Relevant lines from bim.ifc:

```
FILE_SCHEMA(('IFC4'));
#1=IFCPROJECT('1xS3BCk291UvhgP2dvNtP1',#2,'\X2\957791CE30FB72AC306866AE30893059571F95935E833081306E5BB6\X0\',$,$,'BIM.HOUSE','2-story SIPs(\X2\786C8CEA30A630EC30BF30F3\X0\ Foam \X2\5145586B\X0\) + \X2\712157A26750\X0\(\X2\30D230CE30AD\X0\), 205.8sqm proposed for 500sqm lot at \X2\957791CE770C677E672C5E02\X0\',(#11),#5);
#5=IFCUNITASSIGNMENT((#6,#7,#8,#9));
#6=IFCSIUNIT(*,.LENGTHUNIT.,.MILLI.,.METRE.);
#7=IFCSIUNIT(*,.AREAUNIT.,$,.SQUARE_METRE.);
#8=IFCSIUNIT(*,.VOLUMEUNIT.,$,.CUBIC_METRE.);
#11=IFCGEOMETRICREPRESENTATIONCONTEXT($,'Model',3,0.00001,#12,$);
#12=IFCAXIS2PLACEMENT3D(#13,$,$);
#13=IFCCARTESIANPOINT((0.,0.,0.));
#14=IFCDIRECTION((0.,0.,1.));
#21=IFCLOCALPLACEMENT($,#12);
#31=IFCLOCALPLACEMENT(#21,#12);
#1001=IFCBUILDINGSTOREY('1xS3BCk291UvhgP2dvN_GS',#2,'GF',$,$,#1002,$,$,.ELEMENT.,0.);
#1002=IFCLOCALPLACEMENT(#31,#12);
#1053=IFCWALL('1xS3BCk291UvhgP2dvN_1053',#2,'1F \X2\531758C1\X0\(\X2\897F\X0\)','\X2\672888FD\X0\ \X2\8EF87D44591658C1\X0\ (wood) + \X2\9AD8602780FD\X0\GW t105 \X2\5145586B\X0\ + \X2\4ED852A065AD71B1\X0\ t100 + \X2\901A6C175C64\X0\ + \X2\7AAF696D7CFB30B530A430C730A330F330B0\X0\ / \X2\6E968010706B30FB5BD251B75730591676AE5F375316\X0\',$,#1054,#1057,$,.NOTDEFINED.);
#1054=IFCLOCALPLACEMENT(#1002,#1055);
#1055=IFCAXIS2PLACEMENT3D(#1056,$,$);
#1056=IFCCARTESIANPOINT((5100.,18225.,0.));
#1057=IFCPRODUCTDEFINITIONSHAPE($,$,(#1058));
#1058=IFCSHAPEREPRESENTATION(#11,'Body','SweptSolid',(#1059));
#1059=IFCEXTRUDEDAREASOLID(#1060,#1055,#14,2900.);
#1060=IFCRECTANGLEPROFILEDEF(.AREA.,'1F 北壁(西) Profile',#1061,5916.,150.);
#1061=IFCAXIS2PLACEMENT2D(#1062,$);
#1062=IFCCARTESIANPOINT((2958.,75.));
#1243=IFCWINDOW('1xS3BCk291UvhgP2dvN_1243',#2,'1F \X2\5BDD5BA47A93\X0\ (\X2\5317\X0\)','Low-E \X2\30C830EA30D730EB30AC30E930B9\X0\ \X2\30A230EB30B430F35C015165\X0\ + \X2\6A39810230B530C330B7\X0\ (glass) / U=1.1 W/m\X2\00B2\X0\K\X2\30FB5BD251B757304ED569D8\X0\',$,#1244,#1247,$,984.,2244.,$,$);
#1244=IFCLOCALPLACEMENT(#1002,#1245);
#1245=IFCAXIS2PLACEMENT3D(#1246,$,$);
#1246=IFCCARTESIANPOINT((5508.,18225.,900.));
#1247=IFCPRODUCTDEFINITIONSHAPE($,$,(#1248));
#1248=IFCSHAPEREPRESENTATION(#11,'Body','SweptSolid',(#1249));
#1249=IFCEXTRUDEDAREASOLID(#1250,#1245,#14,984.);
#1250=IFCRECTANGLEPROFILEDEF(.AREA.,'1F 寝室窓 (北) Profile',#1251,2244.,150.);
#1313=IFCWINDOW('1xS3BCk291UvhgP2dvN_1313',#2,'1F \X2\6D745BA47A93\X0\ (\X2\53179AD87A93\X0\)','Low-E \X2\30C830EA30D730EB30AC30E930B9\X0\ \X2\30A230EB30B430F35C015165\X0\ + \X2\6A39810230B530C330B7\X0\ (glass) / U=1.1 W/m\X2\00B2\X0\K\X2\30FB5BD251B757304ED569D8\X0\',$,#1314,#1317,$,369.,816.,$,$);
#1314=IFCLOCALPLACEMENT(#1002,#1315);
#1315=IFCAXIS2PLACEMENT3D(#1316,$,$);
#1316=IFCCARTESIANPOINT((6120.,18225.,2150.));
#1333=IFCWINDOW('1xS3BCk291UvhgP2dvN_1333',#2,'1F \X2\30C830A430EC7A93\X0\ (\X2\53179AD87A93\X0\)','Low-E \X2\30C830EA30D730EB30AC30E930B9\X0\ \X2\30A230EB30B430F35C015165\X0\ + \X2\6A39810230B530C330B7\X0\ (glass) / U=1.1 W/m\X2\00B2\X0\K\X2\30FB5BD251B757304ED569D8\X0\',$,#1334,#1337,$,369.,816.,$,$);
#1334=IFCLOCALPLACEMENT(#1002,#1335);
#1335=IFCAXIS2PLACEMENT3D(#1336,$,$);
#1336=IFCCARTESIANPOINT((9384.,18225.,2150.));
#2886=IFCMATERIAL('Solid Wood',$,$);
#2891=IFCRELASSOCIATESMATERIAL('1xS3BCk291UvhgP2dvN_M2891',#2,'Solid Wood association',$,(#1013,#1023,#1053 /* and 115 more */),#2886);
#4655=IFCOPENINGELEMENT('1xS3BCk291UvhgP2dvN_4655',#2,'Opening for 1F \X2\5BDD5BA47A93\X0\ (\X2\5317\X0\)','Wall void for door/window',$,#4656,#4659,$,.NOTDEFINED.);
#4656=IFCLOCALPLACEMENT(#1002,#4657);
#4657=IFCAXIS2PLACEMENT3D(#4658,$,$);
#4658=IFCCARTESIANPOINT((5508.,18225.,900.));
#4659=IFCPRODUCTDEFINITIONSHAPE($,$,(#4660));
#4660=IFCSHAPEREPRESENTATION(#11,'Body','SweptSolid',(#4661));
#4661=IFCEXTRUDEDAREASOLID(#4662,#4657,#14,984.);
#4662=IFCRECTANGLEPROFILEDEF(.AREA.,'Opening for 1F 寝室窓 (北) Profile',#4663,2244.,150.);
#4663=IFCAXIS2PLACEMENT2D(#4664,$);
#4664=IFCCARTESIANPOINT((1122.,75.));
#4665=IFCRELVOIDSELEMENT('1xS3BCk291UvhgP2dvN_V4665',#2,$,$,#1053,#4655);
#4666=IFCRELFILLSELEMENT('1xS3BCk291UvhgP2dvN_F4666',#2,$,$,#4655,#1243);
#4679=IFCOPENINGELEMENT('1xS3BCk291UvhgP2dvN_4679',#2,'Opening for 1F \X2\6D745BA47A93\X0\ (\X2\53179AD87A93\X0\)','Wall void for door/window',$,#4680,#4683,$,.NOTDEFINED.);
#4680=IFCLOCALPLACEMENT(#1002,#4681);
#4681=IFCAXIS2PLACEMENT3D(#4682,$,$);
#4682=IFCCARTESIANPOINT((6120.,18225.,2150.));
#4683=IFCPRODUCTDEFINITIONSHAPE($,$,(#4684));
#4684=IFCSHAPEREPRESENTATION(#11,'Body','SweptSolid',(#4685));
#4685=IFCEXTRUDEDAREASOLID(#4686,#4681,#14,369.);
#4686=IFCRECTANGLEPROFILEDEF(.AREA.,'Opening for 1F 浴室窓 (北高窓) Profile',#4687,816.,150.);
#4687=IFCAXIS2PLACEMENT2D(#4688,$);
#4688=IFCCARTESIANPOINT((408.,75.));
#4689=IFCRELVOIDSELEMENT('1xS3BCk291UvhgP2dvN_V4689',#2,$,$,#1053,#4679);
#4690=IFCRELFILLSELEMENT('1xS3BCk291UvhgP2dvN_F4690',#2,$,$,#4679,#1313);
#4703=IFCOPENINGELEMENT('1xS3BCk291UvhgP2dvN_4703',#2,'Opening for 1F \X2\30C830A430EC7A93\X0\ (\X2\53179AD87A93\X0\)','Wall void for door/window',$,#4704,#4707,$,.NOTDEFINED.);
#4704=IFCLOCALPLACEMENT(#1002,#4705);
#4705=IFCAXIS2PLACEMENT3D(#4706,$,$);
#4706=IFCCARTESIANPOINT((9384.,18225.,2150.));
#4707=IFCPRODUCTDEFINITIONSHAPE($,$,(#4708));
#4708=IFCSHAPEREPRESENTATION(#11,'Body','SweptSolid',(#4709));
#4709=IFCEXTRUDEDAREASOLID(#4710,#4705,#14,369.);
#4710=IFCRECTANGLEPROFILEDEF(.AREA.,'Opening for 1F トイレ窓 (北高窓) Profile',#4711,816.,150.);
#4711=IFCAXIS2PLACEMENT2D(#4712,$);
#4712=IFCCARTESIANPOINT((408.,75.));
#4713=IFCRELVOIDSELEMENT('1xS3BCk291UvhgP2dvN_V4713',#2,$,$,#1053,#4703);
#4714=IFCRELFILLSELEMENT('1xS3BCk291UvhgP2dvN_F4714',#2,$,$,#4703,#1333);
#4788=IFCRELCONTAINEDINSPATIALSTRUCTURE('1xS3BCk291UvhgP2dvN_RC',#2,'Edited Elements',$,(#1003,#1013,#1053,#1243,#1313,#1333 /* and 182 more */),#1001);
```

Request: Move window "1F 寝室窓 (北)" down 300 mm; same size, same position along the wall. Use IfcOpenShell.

```python
import numpy as np
import ifcopenshell
import ifcopenshell.api.geometry
import ifcopenshell.util.placement
import ifcopenshell.util.unit

model = ifcopenshell.open("bim.ifc")
unit_scale = ifcopenshell.util.unit.calculate_unit_scale(model)

window = model.by_guid("1xS3BCk291UvhgP2dvN_1243")
opening = window.FillsVoids[0].RelatingOpeningElement
dz = -300.0

shift = np.array([0.0, 0.0, dz])
# The window is not placed relative to its opening, so move both.
for product in (opening, window):
    matrix = ifcopenshell.util.placement.get_local_placement(product.ObjectPlacement)
    matrix[:3, 3] += shift
    ifcopenshell.api.geometry.edit_object_placement(model, product=product, matrix=matrix, is_si=False)

print(f"moved by {dz * unit_scale:+.3f} m")

model.write("bim_v2.ifc")
```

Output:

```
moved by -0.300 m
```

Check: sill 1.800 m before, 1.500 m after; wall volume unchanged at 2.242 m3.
